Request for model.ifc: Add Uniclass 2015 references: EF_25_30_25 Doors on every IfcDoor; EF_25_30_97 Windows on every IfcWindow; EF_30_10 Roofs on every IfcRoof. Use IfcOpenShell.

First a look at what the model holds.

```python
import ifcopenshell

model = ifcopenshell.open("model.ifc")
print(model.schema)
print("classifications:", [c.Name for c in model.by_type("IfcClassification")])
for ifc_class in ("IfcDoor", "IfcRoof", "IfcStair", "IfcWall", "IfcWindow"):
    print(ifc_class, len(model.by_type(ifc_class)))
```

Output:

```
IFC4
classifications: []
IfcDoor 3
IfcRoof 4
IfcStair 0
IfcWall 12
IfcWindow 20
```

```python
import ifcopenshell
import ifcopenshell.api.classification

model = ifcopenshell.open("model.ifc")

system = ifcopenshell.api.classification.add_classification(model, classification="Uniclass 2015")

codes = {
    "IfcDoor": ("EF_25_30_25", "Doors"),
    "IfcWindow": ("EF_25_30_97", "Windows"),
    "IfcRoof": ("EF_30_10", "Roofs"),
}
for ifc_class, (code, name) in codes.items():
    products = model.by_type(ifc_class)
    ifcopenshell.api.classification.add_reference(
        model, products=products, classification=system, identification=code, name=name
    )
    print(code, len(products))

model.write("model_edited.ifc")
```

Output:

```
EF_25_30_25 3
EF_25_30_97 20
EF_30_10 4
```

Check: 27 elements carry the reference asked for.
